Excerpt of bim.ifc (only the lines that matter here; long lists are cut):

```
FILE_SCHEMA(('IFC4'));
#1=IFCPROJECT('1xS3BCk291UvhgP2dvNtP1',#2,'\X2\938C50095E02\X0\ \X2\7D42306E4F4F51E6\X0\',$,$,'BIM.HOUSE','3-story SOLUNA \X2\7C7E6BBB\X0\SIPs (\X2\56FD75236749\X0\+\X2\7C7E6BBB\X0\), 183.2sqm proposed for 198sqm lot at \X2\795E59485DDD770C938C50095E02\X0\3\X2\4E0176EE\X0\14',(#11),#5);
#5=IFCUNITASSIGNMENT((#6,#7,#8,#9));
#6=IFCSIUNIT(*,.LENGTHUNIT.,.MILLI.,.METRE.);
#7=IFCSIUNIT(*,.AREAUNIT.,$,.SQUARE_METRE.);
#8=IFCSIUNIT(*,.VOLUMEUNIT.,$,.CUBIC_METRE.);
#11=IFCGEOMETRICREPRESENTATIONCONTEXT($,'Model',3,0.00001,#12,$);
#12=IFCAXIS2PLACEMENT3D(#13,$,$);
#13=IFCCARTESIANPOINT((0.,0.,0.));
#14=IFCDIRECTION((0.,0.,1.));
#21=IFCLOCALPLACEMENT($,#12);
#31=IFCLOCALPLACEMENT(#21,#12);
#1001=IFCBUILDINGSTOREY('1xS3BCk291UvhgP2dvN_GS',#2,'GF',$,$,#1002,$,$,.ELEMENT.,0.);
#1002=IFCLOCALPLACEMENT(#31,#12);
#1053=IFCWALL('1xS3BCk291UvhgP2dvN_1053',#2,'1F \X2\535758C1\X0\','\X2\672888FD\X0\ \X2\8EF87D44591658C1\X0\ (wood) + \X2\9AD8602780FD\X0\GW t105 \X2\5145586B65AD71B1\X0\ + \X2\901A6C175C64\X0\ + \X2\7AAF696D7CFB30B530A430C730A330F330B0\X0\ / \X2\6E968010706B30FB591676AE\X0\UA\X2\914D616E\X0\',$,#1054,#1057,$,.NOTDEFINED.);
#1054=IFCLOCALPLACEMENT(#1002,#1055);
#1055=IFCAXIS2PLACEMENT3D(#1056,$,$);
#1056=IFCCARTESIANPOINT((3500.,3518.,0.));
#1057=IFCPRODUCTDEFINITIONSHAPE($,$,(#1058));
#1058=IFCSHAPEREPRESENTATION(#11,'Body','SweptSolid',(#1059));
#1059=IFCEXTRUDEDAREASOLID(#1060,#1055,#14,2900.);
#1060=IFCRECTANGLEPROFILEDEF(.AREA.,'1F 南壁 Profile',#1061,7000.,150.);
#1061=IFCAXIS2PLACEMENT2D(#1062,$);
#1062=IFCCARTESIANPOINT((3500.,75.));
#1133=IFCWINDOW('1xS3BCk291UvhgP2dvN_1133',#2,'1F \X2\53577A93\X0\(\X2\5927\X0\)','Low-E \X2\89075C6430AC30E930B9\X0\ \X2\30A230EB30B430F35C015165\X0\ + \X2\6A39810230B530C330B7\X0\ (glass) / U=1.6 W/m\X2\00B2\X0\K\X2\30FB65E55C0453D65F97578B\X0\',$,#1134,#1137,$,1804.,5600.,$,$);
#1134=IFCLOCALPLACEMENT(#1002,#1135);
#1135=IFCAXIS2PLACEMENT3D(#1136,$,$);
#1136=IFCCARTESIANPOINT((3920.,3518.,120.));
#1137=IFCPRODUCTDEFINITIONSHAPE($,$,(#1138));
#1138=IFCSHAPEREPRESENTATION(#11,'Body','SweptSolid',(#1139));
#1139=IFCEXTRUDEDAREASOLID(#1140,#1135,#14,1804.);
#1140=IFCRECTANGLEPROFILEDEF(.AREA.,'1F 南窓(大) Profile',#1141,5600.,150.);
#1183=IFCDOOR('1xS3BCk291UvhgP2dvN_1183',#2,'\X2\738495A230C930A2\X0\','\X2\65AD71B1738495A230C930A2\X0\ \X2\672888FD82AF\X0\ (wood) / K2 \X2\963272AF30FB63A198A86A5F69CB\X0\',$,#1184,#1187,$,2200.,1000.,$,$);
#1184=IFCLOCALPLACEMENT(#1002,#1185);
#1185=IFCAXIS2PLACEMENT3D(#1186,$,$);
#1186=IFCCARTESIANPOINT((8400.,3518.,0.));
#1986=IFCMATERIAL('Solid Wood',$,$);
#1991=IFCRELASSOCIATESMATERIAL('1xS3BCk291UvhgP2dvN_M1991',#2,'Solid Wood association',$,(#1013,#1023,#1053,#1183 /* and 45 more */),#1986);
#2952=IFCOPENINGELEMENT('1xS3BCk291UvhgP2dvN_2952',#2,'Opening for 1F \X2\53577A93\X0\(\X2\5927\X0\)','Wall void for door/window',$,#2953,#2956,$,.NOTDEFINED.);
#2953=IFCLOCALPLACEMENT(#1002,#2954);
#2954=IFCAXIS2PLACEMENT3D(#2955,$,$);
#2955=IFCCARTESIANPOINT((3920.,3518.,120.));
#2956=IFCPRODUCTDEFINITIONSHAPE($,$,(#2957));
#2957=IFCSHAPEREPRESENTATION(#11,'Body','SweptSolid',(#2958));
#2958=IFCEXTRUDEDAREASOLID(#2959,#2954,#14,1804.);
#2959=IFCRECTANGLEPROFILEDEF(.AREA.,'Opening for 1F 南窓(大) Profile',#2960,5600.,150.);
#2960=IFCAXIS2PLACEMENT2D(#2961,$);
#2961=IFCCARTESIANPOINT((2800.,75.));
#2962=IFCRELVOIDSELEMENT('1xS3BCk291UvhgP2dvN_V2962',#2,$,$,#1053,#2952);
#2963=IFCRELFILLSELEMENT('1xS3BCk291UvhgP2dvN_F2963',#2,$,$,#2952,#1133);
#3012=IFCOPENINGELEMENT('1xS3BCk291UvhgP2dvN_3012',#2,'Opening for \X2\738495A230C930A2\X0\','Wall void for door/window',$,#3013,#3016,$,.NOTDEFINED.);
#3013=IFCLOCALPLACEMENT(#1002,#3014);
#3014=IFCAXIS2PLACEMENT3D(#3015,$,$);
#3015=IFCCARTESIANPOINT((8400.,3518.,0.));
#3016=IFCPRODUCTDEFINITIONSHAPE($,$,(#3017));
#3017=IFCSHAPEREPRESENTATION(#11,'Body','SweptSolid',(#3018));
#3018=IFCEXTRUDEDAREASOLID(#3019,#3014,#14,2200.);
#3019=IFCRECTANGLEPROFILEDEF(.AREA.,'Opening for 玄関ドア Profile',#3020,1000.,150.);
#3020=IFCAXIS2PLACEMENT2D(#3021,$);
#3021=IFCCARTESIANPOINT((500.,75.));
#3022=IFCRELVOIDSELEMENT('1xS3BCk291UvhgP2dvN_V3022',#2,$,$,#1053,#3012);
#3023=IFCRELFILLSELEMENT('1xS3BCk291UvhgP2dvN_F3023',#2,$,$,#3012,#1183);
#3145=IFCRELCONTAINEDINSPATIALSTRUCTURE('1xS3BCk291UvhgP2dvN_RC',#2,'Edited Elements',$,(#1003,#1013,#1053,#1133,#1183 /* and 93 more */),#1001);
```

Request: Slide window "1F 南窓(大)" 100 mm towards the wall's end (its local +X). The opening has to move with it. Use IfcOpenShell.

```python
import ifcopenshell
import ifcopenshell.api.geometry
import ifcopenshell.util.placement
import ifcopenshell.util.unit

model = ifcopenshell.open("bim.ifc")
unit_scale = ifcopenshell.util.unit.calculate_unit_scale(model)

window = model.by_guid("1xS3BCk291UvhgP2dvN_1133")
opening = window.FillsVoids[0].RelatingOpeningElement
wall = opening.VoidsElements[0].RelatingBuildingElement

wall_matrix = ifcopenshell.util.placement.get_local_placement(wall.ObjectPlacement)
shift = wall_matrix[:3, 0] * 0.1 / unit_scale
before = ifcopenshell.util.placement.get_local_placement(window.ObjectPlacement)[:3, 3].copy()

# The window is not placed relative to its opening, so move both.
for product in (opening, window):
    matrix = ifcopenshell.util.placement.get_local_placement(product.ObjectPlacement)
    matrix[:3, 3] += shift
    ifcopenshell.api.geometry.edit_object_placement(model, product=product, matrix=matrix, is_si=False)

after = ifcopenshell.util.placement.get_local_placement(window.ObjectPlacement)[:3, 3]
print("window moved by", (after - before).round(3) + 0.0)

model.write("bim_updated.ifc")
```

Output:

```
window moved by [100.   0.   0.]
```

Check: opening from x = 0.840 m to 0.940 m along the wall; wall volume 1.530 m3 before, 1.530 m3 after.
